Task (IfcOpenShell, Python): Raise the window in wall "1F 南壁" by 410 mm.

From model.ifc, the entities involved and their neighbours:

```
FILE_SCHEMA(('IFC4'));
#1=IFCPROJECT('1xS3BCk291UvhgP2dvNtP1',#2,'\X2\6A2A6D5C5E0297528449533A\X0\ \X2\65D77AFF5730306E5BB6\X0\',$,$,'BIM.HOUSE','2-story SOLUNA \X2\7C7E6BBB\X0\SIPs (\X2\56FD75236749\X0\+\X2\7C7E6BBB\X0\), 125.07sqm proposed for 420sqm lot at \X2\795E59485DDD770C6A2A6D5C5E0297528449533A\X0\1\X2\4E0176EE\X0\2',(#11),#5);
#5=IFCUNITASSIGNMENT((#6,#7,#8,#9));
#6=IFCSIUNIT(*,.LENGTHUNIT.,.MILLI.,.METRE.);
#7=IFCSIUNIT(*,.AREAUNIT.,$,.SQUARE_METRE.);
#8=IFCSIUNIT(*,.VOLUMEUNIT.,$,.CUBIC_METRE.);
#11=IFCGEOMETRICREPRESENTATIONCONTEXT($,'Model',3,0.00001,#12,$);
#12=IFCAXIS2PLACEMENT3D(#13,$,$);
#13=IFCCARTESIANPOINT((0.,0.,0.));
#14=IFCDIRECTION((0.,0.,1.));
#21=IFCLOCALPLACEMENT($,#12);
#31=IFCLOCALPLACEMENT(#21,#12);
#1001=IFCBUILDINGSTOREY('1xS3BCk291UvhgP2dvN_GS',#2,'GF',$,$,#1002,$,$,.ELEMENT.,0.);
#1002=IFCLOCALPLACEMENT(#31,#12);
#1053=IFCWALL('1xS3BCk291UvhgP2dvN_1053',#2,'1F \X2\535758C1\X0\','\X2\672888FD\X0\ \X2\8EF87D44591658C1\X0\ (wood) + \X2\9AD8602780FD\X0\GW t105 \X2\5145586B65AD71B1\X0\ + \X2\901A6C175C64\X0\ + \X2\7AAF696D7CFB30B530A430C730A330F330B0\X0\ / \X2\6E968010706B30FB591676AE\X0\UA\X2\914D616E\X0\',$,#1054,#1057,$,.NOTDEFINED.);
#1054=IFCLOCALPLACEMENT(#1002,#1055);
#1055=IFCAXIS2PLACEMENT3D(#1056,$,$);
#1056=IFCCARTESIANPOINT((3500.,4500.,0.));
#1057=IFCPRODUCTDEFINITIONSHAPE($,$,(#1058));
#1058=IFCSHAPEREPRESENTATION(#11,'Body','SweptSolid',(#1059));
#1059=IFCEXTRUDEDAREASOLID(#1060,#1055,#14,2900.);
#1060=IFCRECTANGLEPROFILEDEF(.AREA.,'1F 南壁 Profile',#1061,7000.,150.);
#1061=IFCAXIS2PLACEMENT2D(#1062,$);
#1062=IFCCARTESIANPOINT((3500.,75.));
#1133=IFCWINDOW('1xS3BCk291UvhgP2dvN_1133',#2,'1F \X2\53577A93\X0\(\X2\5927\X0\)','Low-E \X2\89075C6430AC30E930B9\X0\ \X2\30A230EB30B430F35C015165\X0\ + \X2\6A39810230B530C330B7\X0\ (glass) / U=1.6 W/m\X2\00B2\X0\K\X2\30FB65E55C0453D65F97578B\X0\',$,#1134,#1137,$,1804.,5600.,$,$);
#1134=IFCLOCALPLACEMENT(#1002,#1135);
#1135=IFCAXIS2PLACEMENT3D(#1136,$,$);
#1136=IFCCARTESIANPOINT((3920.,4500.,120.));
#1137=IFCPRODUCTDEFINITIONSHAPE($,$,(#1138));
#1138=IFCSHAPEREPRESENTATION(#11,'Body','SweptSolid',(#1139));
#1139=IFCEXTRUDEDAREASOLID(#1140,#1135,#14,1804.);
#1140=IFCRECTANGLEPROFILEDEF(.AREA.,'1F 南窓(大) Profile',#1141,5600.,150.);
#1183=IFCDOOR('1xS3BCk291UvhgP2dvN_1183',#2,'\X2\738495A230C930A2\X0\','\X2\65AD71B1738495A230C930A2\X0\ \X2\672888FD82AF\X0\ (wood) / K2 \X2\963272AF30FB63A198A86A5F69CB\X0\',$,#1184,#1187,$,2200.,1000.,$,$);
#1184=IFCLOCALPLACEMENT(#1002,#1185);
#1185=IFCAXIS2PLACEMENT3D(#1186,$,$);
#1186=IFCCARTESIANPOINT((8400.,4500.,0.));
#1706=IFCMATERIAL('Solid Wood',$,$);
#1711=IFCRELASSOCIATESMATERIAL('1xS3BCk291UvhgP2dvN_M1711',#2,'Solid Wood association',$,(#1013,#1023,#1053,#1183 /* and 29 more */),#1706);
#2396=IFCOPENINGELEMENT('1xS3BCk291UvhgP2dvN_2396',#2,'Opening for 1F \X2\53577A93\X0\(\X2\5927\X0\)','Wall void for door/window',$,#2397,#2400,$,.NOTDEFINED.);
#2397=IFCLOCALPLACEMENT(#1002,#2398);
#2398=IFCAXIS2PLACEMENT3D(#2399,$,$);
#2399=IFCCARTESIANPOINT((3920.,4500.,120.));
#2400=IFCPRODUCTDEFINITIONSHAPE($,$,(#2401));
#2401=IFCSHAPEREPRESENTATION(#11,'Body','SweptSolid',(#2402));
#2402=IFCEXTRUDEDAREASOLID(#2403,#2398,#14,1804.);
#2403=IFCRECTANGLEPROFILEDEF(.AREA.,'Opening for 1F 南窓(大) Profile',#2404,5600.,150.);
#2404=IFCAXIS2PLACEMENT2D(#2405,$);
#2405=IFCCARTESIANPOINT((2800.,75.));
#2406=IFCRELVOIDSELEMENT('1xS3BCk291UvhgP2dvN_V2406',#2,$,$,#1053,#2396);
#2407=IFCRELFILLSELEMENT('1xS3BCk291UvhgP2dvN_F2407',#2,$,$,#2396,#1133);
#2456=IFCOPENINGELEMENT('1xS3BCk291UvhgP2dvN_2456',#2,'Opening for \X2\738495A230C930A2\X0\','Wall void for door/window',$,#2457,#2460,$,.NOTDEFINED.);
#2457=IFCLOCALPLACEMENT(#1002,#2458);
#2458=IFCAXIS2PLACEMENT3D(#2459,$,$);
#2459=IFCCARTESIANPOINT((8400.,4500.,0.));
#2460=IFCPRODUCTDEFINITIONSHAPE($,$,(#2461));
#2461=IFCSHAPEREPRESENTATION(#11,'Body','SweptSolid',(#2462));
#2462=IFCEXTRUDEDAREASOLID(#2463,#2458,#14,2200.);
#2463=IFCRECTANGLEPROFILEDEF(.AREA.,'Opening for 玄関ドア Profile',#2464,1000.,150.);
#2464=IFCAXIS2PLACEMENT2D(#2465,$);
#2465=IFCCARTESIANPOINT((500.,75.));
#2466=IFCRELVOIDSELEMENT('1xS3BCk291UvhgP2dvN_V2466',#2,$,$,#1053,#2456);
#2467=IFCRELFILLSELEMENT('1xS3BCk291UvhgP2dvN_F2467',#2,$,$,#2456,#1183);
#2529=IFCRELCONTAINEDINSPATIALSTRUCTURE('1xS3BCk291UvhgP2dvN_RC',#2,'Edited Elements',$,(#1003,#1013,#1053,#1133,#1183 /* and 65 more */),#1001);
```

```python
import numpy as np
import ifcopenshell
import ifcopenshell.api.geometry
import ifcopenshell.util.placement
import ifcopenshell.util.unit

model = ifcopenshell.open("model.ifc")
unit_scale = ifcopenshell.util.unit.calculate_unit_scale(model)

window = model.by_guid("1xS3BCk291UvhgP2dvN_1133")
opening = window.FillsVoids[0].RelatingOpeningElement
dz = 410.0

shift = np.array([0.0, 0.0, dz])
# The window is not placed relative to its opening, so move both.
for product in (opening, window):
    matrix = ifcopenshell.util.placement.get_local_placement(product.ObjectPlacement)
    matrix[:3, 3] += shift
    ifcopenshell.api.geometry.edit_object_placement(model, product=product, matrix=matrix, is_si=False)

print(f"moved by {dz * unit_scale:+.3f} m")

model.write("model_updated.ifc")
```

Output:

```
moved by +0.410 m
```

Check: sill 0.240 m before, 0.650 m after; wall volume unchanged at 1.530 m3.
